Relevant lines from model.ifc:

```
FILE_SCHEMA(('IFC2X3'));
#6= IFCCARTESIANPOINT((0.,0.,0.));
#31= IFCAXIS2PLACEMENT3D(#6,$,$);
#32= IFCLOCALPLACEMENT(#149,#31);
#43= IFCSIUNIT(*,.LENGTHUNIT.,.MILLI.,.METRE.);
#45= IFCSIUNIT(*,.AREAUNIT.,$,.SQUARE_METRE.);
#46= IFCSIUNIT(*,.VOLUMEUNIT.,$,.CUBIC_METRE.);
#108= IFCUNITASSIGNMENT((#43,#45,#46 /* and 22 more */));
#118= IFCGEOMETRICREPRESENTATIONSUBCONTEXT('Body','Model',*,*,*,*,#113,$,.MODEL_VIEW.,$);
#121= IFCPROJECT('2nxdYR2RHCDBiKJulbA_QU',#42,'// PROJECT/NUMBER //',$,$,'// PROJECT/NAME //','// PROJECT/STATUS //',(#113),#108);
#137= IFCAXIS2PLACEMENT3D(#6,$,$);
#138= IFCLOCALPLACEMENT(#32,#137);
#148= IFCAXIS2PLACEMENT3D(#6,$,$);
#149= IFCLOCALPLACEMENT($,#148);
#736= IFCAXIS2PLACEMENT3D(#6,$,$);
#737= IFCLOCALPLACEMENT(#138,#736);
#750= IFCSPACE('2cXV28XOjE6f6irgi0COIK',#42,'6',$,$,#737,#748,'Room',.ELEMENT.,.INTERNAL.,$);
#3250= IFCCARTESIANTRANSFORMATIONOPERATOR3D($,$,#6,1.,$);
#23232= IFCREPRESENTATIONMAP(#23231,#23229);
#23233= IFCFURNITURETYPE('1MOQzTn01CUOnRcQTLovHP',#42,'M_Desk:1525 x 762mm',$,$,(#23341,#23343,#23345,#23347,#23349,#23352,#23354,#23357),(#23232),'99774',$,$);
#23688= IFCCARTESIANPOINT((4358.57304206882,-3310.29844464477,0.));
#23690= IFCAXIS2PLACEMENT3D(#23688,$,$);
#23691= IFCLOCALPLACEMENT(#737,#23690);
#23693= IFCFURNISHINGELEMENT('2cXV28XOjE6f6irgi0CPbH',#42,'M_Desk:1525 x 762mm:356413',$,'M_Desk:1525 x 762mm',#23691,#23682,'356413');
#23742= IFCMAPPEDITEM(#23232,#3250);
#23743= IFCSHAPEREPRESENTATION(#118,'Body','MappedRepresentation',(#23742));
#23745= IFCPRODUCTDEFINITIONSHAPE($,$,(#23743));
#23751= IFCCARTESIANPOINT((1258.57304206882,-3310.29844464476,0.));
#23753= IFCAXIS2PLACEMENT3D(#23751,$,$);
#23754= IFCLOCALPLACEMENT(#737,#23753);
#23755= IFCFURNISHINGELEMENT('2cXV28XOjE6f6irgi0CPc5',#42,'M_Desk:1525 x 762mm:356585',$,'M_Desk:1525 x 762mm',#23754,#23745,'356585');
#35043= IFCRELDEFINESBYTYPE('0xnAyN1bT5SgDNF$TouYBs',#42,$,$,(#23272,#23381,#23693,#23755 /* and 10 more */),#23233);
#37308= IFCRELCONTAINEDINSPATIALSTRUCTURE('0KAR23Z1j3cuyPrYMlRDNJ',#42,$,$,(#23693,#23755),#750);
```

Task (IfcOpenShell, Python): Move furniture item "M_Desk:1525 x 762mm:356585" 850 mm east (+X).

```python
import ifcopenshell
import ifcopenshell.api.geometry
import ifcopenshell.util.placement
import ifcopenshell.util.unit

model = ifcopenshell.open("model.ifc")
unit_scale = ifcopenshell.util.unit.calculate_unit_scale(model)

item = model.by_id(23755)
matrix = ifcopenshell.util.placement.get_local_placement(item.ObjectPlacement)
matrix[0, 3] += 0.85 / unit_scale
ifcopenshell.api.geometry.edit_object_placement(model, product=item, matrix=matrix, is_si=False)

print(ifcopenshell.util.placement.get_local_placement(item.ObjectPlacement).round(3) + 0.0)

model.write("model_v2.ifc")
```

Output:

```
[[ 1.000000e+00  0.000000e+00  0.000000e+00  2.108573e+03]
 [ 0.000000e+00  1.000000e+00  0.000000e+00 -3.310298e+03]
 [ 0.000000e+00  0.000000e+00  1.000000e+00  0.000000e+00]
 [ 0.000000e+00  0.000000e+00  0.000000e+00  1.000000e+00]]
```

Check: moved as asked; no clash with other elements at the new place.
